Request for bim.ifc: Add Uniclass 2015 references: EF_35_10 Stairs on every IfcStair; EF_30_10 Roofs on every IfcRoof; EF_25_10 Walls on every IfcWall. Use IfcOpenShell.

First a look at what the model holds.

```python
import ifcopenshell

model = ifcopenshell.open("bim.ifc")
print(model.schema)
print("classifications:", [c.Name for c in model.by_type("IfcClassification")])
for ifc_class in ("IfcDoor", "IfcRoof", "IfcStair", "IfcWall", "IfcWindow"):
    print(ifc_class, len(model.by_type(ifc_class)))
```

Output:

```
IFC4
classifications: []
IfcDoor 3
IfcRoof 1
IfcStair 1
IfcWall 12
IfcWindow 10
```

```python
import ifcopenshell
import ifcopenshell.api.classification

model = ifcopenshell.open("bim.ifc")

system = ifcopenshell.api.classification.add_classification(model, classification="Uniclass 2015")

codes = {
    "IfcStair": ("EF_35_10", "Stairs"),
    "IfcRoof": ("EF_30_10", "Roofs"),
    "IfcWall": ("EF_25_10", "Walls"),
}
for ifc_class, (code, name) in codes.items():
    products = model.by_type(ifc_class)
    ifcopenshell.api.classification.add_reference(
        model, products=products, classification=system, identification=code, name=name
    )
    print(code, len(products))

model.write("bim_updated.ifc")
```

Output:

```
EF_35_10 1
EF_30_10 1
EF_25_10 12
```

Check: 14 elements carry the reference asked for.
